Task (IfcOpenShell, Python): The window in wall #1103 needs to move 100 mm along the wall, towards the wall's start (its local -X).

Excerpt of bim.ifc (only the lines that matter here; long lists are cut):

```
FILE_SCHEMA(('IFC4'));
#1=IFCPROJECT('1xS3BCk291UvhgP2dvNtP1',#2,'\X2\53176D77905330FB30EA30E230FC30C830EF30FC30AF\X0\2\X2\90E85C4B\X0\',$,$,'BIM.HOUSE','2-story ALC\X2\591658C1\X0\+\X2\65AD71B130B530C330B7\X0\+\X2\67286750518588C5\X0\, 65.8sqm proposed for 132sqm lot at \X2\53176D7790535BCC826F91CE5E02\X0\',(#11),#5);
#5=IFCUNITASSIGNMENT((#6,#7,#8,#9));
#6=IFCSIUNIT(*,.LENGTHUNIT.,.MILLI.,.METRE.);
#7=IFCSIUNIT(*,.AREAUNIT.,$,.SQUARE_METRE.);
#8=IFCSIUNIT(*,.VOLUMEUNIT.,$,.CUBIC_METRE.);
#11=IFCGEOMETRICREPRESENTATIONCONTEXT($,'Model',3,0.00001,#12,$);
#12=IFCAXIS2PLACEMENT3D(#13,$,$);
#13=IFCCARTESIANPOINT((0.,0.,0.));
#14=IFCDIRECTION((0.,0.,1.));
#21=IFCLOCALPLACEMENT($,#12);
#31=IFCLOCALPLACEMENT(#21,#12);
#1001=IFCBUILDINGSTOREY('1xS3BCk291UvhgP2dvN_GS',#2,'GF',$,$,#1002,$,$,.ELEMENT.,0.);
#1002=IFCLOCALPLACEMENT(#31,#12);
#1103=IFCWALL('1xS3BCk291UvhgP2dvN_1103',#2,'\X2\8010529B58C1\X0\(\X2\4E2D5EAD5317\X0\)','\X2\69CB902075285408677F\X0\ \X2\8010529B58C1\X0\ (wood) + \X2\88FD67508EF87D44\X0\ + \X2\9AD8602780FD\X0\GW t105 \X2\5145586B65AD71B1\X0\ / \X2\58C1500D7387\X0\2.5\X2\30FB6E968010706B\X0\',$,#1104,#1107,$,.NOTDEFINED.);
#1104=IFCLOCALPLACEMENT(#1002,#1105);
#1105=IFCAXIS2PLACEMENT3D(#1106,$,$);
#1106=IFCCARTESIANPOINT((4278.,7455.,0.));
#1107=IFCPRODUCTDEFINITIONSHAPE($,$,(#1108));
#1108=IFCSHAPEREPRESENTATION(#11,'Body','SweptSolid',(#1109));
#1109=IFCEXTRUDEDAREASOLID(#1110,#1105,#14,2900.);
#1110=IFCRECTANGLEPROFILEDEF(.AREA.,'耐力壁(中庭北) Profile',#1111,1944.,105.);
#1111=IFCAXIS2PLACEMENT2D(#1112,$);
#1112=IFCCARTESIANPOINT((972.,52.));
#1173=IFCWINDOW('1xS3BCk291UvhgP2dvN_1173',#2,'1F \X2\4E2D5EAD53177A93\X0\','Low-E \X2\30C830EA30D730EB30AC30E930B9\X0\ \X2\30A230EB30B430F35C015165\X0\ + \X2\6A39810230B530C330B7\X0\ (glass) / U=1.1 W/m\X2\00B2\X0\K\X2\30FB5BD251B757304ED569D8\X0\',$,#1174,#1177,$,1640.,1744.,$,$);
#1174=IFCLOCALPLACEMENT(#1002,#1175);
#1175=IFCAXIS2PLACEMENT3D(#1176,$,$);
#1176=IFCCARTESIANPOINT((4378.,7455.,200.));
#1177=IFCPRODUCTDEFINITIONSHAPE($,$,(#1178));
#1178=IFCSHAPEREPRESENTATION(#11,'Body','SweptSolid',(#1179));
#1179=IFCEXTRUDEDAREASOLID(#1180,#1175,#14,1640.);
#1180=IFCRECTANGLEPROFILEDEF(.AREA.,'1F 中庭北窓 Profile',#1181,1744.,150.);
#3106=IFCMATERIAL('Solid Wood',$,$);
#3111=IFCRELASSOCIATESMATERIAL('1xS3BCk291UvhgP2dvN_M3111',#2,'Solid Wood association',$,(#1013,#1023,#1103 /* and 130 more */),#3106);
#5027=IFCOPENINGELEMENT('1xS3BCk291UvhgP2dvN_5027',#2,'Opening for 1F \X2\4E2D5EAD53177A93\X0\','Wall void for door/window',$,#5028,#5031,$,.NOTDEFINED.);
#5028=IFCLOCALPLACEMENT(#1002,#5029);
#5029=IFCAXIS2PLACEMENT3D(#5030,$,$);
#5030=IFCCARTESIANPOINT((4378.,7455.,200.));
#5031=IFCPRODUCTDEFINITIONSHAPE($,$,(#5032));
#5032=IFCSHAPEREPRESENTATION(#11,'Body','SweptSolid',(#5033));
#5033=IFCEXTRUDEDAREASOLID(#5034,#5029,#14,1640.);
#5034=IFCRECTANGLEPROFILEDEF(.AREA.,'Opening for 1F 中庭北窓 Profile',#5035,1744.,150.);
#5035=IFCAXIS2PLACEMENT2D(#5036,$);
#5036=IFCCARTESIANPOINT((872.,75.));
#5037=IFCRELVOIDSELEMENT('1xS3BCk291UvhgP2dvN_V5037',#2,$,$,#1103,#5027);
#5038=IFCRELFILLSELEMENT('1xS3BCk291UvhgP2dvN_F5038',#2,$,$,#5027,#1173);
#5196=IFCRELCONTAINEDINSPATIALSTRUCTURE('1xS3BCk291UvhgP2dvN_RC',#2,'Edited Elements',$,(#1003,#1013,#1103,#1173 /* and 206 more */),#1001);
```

```python
import ifcopenshell
import ifcopenshell.api.geometry
import ifcopenshell.util.placement
import ifcopenshell.util.unit

model = ifcopenshell.open("bim.ifc")
unit_scale = ifcopenshell.util.unit.calculate_unit_scale(model)

window = model.by_guid("1xS3BCk291UvhgP2dvN_1173")
opening = window.FillsVoids[0].RelatingOpeningElement
wall = opening.VoidsElements[0].RelatingBuildingElement

wall_matrix = ifcopenshell.util.placement.get_local_placement(wall.ObjectPlacement)
shift = wall_matrix[:3, 0] * -0.1 / unit_scale
before = ifcopenshell.util.placement.get_local_placement(window.ObjectPlacement)[:3, 3].copy()

# The window is not placed relative to its opening, so move both.
for product in (opening, window):
    matrix = ifcopenshell.util.placement.get_local_placement(product.ObjectPlacement)
    matrix[:3, 3] += shift
    ifcopenshell.api.geometry.edit_object_placement(model, product=product, matrix=matrix, is_si=False)

after = ifcopenshell.util.placement.get_local_placement(window.ObjectPlacement)[:3, 3]
print("window moved by", (after - before).round(3) + 0.0)

model.write("bim-out.ifc")
```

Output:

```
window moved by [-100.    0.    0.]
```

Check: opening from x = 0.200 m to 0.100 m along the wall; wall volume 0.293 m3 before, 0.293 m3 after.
